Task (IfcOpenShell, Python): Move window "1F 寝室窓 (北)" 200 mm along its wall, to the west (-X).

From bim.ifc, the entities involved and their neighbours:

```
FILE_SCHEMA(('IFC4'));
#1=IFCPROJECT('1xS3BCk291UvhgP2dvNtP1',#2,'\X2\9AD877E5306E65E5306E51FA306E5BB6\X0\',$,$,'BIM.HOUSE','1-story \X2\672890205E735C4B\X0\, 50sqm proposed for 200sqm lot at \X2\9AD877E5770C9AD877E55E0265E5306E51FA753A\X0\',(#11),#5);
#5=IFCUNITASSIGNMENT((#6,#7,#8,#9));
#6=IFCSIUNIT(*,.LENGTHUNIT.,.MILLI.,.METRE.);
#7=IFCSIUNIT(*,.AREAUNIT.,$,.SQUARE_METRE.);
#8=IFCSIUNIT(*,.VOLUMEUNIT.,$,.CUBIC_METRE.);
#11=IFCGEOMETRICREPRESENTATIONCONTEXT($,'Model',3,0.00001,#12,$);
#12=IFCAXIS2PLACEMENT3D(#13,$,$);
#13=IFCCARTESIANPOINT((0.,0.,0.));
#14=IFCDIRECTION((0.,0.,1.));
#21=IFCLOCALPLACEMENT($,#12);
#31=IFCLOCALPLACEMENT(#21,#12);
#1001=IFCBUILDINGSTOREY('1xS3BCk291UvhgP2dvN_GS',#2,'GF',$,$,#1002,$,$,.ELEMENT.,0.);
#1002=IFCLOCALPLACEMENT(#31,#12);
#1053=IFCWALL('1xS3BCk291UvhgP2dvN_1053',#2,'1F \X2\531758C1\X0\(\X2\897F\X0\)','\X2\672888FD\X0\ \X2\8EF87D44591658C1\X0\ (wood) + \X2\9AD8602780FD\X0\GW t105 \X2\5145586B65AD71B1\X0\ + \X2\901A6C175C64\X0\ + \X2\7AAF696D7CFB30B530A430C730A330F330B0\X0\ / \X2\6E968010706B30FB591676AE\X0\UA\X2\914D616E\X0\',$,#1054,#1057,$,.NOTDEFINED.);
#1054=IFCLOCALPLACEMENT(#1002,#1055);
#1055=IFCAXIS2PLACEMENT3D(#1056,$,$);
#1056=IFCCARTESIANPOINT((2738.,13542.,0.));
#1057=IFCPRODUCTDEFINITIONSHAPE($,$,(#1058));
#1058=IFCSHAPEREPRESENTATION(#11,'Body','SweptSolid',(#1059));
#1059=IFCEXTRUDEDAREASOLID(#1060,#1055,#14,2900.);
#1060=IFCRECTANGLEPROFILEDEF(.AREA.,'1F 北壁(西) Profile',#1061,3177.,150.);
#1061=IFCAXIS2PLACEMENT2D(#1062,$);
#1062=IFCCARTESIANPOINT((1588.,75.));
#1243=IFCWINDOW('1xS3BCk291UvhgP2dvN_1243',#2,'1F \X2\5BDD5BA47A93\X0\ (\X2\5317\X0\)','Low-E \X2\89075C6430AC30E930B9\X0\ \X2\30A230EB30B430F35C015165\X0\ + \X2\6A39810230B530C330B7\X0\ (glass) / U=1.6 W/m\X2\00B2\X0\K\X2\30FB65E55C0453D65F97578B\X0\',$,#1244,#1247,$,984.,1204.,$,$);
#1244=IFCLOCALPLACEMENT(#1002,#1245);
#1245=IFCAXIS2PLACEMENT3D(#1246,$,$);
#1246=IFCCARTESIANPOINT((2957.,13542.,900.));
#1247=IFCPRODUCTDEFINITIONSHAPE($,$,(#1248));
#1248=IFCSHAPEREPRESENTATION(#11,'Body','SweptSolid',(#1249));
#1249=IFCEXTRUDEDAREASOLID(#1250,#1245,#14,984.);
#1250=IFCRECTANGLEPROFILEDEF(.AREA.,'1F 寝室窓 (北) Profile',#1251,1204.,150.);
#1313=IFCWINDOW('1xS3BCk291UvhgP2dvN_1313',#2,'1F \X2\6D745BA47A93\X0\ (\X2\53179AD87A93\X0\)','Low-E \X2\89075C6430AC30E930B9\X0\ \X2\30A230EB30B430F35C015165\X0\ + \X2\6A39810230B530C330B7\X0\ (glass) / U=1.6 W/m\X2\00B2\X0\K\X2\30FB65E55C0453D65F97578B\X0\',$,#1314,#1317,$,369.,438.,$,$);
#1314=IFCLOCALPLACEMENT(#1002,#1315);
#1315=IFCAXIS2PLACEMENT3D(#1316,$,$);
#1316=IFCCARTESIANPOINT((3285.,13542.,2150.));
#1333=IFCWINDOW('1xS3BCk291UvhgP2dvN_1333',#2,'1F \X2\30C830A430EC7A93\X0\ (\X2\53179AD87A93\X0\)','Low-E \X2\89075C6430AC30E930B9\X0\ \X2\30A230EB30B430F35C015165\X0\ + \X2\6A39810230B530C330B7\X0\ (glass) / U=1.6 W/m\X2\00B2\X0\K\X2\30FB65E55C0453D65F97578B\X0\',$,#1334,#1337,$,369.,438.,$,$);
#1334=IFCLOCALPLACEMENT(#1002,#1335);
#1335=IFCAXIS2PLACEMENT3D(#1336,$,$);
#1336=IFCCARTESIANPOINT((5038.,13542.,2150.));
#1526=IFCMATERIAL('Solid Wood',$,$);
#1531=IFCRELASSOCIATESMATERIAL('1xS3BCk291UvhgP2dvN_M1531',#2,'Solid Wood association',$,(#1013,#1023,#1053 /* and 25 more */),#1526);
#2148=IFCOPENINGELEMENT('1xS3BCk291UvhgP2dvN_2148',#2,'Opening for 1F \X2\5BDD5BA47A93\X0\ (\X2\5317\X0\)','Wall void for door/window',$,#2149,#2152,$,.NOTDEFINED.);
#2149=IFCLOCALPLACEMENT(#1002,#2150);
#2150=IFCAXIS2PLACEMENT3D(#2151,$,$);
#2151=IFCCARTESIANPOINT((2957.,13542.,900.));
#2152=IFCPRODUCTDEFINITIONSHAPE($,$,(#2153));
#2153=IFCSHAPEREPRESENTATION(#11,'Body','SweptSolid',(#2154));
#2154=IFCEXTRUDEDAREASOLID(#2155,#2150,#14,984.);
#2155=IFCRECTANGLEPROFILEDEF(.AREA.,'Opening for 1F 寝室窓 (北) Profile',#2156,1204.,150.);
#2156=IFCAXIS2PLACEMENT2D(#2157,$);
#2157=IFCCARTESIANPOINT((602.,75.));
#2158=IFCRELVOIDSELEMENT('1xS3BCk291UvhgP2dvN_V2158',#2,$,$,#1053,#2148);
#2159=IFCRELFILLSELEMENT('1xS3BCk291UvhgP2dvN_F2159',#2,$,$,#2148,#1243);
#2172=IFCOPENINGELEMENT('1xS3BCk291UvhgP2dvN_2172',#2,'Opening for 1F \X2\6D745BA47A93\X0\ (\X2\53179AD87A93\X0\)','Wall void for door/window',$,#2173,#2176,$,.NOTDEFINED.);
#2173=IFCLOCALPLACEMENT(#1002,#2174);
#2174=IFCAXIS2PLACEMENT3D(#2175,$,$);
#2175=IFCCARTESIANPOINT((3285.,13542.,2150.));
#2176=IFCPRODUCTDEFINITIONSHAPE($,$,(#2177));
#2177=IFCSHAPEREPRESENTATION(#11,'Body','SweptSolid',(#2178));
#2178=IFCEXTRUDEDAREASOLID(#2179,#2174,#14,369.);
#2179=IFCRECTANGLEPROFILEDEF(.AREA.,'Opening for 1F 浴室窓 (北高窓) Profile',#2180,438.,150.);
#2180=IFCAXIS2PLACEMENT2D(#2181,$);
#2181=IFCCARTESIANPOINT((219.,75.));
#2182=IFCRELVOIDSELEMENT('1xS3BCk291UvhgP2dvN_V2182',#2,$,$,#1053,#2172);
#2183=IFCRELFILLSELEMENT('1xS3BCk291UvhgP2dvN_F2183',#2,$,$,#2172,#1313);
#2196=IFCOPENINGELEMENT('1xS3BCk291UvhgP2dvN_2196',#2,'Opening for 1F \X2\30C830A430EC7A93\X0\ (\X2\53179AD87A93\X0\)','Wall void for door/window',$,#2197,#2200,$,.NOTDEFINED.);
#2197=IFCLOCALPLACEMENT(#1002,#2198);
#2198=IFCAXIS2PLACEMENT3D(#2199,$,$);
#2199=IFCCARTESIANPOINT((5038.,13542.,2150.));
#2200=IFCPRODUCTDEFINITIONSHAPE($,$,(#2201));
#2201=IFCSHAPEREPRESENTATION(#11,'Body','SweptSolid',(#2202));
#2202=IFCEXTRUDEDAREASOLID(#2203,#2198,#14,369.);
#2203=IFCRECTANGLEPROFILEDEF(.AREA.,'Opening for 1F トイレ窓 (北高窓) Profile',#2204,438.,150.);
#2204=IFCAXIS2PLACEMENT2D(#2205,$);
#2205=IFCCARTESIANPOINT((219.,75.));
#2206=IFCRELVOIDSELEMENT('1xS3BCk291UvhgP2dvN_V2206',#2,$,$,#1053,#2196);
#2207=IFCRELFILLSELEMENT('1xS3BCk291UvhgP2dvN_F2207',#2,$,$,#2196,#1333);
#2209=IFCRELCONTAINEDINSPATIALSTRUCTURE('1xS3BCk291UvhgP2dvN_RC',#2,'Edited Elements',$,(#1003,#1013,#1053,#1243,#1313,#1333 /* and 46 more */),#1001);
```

```python
import ifcopenshell
import ifcopenshell.api.geometry
import ifcopenshell.util.placement
import ifcopenshell.util.unit

model = ifcopenshell.open("bim.ifc")
unit_scale = ifcopenshell.util.unit.calculate_unit_scale(model)

window = model.by_id(1243)
opening = window.FillsVoids[0].RelatingOpeningElement
wall = opening.VoidsElements[0].RelatingBuildingElement

wall_matrix = ifcopenshell.util.placement.get_local_placement(wall.ObjectPlacement)
shift = wall_matrix[:3, 0] * -0.2 / unit_scale
before = ifcopenshell.util.placement.get_local_placement(window.ObjectPlacement)[:3, 3].copy()

# The window is not placed relative to its opening, so move both.
for product in (opening, window):
    matrix = ifcopenshell.util.placement.get_local_placement(product.ObjectPlacement)
    matrix[:3, 3] += shift
    ifcopenshell.api.geometry.edit_object_placement(model, product=product, matrix=matrix, is_si=False)

after = ifcopenshell.util.placement.get_local_placement(window.ObjectPlacement)[:3, 3]
print("window moved by", (after - before).round(3) + 0.0)

model.write("bim_updated.ifc")
```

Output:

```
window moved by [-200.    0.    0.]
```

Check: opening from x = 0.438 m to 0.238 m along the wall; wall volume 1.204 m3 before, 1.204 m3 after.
